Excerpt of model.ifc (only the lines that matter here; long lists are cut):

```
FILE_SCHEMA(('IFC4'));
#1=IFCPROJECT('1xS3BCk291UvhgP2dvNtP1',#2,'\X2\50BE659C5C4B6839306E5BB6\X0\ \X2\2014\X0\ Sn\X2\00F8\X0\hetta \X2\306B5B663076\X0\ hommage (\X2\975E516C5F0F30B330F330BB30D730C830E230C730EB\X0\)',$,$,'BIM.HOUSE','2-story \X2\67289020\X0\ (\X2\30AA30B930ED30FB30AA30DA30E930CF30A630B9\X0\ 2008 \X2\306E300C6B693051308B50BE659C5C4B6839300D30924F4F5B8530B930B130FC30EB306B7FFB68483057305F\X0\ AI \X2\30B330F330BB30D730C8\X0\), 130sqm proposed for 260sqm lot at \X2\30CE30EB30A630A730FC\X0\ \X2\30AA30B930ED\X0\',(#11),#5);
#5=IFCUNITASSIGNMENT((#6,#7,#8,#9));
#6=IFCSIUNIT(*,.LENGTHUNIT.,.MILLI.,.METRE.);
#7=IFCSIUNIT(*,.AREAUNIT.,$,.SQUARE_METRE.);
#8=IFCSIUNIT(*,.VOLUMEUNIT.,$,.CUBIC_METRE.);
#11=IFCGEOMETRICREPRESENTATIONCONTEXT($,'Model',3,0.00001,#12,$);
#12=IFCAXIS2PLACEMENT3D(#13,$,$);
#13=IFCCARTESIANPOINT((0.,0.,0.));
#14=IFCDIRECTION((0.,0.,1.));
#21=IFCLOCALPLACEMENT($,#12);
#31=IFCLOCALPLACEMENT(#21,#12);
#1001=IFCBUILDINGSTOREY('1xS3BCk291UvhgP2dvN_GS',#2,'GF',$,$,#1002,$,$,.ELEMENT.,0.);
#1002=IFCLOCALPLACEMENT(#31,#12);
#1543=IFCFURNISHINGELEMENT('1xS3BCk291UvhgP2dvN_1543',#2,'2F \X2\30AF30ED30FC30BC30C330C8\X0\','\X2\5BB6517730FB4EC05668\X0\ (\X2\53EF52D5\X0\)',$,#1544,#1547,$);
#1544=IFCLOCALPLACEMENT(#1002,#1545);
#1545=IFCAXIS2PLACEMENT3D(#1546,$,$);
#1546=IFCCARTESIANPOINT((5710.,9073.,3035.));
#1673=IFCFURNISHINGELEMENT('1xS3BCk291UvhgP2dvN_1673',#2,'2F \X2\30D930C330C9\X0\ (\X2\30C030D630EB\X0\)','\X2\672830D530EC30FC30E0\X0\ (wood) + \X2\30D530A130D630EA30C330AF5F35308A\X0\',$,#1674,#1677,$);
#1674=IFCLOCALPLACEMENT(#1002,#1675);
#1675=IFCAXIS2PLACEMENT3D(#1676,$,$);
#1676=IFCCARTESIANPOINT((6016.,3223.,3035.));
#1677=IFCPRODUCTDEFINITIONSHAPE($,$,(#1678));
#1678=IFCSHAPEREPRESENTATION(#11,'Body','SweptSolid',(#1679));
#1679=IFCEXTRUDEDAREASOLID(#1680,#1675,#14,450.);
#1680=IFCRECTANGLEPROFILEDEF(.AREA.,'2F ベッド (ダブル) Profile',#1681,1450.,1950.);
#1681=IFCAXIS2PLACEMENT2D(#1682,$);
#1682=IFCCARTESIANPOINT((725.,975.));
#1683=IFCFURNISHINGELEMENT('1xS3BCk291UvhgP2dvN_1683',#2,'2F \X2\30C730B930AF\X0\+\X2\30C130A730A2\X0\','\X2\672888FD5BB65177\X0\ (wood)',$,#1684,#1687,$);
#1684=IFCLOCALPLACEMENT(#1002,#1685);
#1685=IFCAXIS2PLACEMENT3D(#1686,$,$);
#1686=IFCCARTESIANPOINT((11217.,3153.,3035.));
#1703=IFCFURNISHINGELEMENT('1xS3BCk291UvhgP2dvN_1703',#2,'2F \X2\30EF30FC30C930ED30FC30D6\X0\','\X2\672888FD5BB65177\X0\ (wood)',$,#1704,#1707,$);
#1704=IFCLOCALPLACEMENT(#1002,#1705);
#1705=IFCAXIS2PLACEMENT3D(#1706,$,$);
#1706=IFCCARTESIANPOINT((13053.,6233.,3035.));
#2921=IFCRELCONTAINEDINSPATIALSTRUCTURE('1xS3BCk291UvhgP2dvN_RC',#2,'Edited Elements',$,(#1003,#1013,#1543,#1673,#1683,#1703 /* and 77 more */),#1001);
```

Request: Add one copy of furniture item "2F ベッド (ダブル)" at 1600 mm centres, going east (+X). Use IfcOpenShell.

```python
import numpy as np
import ifcopenshell
import ifcopenshell.api.geometry
import ifcopenshell.api.root
import ifcopenshell.util.element
import ifcopenshell.util.placement

model = ifcopenshell.open("model.ifc")


def reuse_history(source, copy):
    """copy_class also copies each property set's owner history, people and application; keep the originals."""
    for rel in copy.IsDefinedBy:
        if rel.is_a("IfcRelDefinesByProperties") and (history := rel.RelatingPropertyDefinition.OwnerHistory):
            rel.RelatingPropertyDefinition.OwnerHistory = source.OwnerHistory
            ifcopenshell.util.element.remove_deep2(model, history)


source = model.by_guid("1xS3BCk291UvhgP2dvN_1673")
base = ifcopenshell.util.placement.get_local_placement(source.ObjectPlacement)
step = np.array([1.0, 0.0, 0.0]) * 1600.0

for i in range(1, 2):
    copy = ifcopenshell.api.root.copy_class(model, product=source)
    copy.Representation = ifcopenshell.util.element.copy_deep(
        model, source.Representation, exclude=["IfcGeometricRepresentationContext", "IfcRepresentationMap"]
    )
    reuse_history(source, copy)
    matrix = base.copy()
    matrix[:3, 3] += i * step
    print("added at", matrix[:3, 3].round(3) + 0.0)
    ifcopenshell.api.geometry.edit_object_placement(model, product=copy, matrix=matrix, is_si=False)

model.write("model_rev.ifc")
```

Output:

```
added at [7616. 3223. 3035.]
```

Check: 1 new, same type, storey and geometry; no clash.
